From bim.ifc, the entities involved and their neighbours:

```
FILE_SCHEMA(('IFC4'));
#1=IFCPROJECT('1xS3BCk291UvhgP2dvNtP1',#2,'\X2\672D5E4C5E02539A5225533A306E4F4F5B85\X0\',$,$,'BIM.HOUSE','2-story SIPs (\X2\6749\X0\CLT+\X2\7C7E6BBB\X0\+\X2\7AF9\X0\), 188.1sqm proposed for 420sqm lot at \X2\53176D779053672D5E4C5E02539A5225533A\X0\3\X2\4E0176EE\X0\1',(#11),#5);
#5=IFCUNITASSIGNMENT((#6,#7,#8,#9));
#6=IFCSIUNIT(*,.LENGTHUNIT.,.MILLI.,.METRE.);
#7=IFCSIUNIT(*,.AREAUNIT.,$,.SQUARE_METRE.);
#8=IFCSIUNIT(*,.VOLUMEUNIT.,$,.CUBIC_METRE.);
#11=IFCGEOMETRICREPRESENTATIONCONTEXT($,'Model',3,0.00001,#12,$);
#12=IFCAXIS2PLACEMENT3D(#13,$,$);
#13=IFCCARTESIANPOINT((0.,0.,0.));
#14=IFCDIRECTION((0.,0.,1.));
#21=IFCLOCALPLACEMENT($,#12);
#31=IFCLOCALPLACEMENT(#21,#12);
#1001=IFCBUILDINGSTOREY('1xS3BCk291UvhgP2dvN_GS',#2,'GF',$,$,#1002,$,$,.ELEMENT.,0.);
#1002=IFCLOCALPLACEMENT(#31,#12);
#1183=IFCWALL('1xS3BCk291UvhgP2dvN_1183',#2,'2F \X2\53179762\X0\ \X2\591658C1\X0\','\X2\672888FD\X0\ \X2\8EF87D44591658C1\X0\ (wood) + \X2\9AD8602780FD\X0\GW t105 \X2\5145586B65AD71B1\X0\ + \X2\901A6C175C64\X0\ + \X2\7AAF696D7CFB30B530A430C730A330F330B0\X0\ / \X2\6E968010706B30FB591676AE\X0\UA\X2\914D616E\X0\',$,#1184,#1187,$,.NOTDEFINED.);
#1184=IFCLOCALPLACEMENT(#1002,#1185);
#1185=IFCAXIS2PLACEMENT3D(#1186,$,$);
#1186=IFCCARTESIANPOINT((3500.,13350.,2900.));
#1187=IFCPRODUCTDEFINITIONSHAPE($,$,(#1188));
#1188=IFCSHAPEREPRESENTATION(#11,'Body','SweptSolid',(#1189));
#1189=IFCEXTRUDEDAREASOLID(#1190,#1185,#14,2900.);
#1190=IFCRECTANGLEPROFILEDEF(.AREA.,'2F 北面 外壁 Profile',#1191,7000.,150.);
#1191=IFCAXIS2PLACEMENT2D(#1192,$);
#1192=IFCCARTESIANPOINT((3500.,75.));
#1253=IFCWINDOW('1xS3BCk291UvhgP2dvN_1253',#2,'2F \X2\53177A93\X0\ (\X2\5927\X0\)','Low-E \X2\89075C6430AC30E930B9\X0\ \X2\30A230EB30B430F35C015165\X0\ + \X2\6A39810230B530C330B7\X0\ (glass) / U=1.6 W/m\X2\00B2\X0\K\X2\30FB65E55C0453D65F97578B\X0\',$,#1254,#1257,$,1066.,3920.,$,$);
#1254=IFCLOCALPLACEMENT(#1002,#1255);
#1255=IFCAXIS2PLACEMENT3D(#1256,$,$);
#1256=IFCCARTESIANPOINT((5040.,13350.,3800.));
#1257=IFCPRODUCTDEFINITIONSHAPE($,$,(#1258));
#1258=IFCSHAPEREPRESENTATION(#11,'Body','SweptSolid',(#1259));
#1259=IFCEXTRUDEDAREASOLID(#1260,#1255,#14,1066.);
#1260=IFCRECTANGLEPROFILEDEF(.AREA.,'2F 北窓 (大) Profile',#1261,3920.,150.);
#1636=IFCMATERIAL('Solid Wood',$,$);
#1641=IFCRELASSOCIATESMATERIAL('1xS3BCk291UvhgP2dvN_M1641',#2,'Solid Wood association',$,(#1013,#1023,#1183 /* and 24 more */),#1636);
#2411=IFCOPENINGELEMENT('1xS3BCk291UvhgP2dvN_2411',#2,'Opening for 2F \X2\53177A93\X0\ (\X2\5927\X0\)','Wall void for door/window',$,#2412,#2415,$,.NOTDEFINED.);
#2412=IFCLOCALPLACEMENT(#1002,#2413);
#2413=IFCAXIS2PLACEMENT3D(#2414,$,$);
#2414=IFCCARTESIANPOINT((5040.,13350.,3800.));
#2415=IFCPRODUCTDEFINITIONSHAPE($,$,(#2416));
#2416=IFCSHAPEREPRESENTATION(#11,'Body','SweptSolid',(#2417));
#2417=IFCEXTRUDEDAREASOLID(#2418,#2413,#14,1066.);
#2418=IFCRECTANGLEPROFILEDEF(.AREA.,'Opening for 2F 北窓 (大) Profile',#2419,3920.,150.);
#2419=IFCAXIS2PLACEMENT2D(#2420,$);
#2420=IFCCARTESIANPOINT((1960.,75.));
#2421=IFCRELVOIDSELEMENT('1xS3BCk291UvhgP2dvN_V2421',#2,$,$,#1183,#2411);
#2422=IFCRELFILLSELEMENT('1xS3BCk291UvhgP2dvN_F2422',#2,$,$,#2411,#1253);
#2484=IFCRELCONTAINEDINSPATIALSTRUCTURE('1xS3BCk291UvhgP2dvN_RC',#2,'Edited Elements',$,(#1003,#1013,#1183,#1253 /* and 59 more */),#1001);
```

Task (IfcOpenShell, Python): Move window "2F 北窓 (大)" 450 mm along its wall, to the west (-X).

```python
import ifcopenshell
import ifcopenshell.api.geometry
import ifcopenshell.util.placement
import ifcopenshell.util.unit

model = ifcopenshell.open("bim.ifc")
unit_scale = ifcopenshell.util.unit.calculate_unit_scale(model)

window = model.by_id(1253)
opening = window.FillsVoids[0].RelatingOpeningElement
wall = opening.VoidsElements[0].RelatingBuildingElement

wall_matrix = ifcopenshell.util.placement.get_local_placement(wall.ObjectPlacement)
shift = wall_matrix[:3, 0] * -0.45 / unit_scale
before = ifcopenshell.util.placement.get_local_placement(window.ObjectPlacement)[:3, 3].copy()

# The window is not placed relative to its opening, so move both.
for product in (opening, window):
    matrix = ifcopenshell.util.placement.get_local_placement(product.ObjectPlacement)
    matrix[:3, 3] += shift
    ifcopenshell.api.geometry.edit_object_placement(model, product=product, matrix=matrix, is_si=False)

after = ifcopenshell.util.placement.get_local_placement(window.ObjectPlacement)[:3, 3]
print("window moved by", (after - before).round(3) + 0.0)

model.write("bim-out.ifc")
```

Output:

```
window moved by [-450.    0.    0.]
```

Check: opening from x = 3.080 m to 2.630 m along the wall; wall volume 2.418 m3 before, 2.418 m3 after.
